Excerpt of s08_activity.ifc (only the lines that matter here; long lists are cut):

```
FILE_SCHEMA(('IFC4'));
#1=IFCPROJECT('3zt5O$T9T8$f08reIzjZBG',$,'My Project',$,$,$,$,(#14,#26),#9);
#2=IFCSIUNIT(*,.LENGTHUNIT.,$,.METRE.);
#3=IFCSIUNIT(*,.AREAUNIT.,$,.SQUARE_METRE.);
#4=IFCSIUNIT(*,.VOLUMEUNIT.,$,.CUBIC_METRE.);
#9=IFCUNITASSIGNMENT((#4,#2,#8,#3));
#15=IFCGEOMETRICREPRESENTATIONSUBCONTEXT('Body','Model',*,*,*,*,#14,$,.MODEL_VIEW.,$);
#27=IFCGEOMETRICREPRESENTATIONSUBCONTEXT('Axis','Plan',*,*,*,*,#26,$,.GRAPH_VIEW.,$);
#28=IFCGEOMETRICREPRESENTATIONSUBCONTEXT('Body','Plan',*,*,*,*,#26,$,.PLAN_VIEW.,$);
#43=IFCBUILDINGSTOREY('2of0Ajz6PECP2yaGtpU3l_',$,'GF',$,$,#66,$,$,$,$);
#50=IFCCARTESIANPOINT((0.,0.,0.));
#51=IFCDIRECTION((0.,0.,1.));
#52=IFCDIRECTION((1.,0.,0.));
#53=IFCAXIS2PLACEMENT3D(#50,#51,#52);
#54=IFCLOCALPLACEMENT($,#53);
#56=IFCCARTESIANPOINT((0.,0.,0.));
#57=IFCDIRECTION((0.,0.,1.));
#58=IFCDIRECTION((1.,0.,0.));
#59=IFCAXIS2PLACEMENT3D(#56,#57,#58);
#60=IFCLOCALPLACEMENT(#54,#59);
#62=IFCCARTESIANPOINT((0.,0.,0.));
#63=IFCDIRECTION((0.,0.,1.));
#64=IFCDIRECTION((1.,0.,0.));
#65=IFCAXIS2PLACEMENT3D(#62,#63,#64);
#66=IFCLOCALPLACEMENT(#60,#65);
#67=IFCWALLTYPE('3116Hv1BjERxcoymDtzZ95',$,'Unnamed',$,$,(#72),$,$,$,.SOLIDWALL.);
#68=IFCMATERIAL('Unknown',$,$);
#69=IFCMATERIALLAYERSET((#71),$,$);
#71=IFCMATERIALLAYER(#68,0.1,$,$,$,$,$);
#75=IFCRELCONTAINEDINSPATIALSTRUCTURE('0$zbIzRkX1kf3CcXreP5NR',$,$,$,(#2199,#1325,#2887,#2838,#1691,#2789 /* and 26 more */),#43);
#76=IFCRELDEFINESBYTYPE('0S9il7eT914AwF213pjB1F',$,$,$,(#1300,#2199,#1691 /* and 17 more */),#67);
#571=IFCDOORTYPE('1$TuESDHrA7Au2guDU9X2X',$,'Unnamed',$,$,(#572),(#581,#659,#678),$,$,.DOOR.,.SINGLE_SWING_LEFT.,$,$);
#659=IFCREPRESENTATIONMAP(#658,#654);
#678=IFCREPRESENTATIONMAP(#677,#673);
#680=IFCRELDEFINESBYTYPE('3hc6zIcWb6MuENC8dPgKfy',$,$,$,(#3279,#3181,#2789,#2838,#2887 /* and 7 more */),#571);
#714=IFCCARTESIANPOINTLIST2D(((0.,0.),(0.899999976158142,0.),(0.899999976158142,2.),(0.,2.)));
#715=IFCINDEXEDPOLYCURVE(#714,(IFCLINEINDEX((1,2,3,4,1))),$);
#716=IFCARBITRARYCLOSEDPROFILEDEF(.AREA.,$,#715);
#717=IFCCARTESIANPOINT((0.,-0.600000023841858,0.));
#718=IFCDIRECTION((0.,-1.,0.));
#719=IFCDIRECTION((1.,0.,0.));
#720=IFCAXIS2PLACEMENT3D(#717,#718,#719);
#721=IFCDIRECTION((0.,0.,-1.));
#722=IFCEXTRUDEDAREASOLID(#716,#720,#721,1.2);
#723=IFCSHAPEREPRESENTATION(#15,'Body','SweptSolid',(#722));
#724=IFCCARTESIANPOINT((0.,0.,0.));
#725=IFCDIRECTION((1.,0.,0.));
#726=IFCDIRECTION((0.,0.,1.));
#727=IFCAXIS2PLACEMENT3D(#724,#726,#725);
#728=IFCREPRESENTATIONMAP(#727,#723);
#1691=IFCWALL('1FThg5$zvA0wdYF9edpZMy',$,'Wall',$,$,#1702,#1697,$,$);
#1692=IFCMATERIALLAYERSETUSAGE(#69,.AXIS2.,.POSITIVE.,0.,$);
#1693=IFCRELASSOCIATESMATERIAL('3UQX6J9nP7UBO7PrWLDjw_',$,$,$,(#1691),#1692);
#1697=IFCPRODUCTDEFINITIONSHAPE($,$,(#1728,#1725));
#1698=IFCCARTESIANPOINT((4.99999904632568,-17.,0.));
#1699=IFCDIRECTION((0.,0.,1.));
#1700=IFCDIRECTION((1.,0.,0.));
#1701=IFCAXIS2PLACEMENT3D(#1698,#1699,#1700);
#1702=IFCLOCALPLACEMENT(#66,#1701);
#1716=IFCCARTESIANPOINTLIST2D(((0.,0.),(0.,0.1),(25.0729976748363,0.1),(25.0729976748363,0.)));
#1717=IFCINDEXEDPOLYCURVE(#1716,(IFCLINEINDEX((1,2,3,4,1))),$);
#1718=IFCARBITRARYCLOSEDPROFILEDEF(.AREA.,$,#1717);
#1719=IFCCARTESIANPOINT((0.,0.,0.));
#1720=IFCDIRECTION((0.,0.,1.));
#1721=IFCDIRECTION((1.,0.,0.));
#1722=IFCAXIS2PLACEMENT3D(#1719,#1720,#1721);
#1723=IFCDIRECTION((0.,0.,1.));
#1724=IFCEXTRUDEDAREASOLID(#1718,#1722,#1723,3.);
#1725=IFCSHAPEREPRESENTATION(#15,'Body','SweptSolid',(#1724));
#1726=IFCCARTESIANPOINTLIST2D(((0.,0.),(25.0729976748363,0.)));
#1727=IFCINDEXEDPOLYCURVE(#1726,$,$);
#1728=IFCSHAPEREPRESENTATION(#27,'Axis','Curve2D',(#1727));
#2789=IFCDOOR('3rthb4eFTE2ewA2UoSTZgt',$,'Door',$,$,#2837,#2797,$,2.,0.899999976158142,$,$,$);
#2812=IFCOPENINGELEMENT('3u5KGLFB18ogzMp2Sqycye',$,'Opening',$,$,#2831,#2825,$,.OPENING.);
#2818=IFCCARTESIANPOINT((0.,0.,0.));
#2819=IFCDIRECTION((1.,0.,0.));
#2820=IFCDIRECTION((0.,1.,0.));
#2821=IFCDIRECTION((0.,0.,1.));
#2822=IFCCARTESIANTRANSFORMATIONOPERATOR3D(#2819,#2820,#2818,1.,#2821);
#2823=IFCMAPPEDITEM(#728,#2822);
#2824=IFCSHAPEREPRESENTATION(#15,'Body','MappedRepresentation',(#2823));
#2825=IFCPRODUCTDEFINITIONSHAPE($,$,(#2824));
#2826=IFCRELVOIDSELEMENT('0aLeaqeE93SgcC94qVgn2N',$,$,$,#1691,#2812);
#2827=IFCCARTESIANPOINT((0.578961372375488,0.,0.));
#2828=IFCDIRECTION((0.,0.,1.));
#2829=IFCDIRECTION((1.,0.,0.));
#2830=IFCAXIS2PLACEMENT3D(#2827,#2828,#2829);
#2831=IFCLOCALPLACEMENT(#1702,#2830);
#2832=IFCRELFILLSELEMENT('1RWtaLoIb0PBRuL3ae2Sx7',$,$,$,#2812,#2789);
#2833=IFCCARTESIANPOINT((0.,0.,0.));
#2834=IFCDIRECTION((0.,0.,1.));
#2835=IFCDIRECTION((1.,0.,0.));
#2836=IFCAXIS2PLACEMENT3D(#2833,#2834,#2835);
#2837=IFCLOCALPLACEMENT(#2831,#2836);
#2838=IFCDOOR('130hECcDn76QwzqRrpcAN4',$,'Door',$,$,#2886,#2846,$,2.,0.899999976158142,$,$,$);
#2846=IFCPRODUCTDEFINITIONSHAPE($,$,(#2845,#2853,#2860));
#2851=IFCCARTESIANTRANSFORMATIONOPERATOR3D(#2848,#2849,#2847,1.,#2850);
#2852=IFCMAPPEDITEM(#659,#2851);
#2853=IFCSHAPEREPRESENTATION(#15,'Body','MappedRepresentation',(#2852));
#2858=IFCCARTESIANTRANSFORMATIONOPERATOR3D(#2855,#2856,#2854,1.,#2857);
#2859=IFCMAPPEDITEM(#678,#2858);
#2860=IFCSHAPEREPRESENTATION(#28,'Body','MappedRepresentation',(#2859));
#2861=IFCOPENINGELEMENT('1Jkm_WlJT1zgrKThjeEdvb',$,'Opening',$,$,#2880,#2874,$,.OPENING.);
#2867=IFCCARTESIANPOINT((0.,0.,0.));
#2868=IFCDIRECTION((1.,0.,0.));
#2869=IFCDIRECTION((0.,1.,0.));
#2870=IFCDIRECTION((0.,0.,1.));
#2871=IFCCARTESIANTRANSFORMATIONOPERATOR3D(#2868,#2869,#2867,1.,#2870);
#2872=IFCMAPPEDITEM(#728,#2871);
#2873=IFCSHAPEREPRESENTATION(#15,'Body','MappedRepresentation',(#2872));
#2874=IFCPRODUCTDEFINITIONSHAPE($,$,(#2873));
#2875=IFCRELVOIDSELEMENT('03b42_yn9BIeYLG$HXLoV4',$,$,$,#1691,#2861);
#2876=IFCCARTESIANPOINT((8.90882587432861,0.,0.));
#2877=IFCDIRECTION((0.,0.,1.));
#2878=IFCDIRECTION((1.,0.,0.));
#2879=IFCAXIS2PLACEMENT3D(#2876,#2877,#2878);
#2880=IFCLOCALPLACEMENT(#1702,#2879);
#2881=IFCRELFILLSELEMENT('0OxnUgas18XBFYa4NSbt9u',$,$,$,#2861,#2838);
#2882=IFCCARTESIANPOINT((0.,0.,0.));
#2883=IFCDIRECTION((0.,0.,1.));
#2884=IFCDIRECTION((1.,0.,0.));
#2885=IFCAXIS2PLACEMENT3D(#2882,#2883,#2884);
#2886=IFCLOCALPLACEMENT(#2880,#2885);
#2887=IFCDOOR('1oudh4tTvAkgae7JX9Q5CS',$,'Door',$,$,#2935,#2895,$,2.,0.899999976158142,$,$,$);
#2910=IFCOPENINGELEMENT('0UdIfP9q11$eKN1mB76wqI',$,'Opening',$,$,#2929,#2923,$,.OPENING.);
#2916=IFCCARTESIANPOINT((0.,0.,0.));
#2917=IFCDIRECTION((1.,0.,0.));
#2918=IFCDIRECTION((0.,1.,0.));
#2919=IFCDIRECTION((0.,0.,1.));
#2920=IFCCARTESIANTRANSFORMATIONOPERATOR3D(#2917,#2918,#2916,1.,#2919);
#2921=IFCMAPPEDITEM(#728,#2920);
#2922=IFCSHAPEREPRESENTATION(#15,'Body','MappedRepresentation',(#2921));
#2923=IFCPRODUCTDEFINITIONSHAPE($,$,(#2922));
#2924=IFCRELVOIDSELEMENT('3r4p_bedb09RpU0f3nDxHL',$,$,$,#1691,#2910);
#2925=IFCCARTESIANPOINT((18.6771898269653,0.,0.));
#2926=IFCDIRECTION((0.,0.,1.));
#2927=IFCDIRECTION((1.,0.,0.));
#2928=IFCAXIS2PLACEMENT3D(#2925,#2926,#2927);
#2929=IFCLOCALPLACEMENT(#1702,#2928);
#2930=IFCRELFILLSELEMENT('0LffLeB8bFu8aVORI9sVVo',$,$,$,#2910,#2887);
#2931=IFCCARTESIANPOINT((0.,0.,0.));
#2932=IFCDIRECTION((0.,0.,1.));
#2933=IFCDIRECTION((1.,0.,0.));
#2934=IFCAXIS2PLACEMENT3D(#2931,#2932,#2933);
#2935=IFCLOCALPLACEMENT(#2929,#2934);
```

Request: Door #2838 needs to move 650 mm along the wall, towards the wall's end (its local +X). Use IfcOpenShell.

```python
import ifcopenshell
import ifcopenshell.api.geometry
import ifcopenshell.util.placement
import ifcopenshell.util.unit

model = ifcopenshell.open("s08_activity.ifc")
unit_scale = ifcopenshell.util.unit.calculate_unit_scale(model)

door = model.by_guid("130hECcDn76QwzqRrpcAN4")
opening = door.FillsVoids[0].RelatingOpeningElement
wall = opening.VoidsElements[0].RelatingBuildingElement

wall_matrix = ifcopenshell.util.placement.get_local_placement(wall.ObjectPlacement)
shift = wall_matrix[:3, 0] * 0.65 / unit_scale
before = ifcopenshell.util.placement.get_local_placement(door.ObjectPlacement)[:3, 3].copy()

# The door is placed relative to its opening, so it follows when the opening moves.
matrix = ifcopenshell.util.placement.get_local_placement(opening.ObjectPlacement)
matrix[:3, 3] += shift
ifcopenshell.api.geometry.edit_object_placement(
    model, product=opening, matrix=matrix, is_si=False, should_transform_children=True
)

after = ifcopenshell.util.placement.get_local_placement(door.ObjectPlacement)[:3, 3]
print("door moved by", (after - before).round(3) + 0.0)

model.write("s08_activity-out.ifc")
```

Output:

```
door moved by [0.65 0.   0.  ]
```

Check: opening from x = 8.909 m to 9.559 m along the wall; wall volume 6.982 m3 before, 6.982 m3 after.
